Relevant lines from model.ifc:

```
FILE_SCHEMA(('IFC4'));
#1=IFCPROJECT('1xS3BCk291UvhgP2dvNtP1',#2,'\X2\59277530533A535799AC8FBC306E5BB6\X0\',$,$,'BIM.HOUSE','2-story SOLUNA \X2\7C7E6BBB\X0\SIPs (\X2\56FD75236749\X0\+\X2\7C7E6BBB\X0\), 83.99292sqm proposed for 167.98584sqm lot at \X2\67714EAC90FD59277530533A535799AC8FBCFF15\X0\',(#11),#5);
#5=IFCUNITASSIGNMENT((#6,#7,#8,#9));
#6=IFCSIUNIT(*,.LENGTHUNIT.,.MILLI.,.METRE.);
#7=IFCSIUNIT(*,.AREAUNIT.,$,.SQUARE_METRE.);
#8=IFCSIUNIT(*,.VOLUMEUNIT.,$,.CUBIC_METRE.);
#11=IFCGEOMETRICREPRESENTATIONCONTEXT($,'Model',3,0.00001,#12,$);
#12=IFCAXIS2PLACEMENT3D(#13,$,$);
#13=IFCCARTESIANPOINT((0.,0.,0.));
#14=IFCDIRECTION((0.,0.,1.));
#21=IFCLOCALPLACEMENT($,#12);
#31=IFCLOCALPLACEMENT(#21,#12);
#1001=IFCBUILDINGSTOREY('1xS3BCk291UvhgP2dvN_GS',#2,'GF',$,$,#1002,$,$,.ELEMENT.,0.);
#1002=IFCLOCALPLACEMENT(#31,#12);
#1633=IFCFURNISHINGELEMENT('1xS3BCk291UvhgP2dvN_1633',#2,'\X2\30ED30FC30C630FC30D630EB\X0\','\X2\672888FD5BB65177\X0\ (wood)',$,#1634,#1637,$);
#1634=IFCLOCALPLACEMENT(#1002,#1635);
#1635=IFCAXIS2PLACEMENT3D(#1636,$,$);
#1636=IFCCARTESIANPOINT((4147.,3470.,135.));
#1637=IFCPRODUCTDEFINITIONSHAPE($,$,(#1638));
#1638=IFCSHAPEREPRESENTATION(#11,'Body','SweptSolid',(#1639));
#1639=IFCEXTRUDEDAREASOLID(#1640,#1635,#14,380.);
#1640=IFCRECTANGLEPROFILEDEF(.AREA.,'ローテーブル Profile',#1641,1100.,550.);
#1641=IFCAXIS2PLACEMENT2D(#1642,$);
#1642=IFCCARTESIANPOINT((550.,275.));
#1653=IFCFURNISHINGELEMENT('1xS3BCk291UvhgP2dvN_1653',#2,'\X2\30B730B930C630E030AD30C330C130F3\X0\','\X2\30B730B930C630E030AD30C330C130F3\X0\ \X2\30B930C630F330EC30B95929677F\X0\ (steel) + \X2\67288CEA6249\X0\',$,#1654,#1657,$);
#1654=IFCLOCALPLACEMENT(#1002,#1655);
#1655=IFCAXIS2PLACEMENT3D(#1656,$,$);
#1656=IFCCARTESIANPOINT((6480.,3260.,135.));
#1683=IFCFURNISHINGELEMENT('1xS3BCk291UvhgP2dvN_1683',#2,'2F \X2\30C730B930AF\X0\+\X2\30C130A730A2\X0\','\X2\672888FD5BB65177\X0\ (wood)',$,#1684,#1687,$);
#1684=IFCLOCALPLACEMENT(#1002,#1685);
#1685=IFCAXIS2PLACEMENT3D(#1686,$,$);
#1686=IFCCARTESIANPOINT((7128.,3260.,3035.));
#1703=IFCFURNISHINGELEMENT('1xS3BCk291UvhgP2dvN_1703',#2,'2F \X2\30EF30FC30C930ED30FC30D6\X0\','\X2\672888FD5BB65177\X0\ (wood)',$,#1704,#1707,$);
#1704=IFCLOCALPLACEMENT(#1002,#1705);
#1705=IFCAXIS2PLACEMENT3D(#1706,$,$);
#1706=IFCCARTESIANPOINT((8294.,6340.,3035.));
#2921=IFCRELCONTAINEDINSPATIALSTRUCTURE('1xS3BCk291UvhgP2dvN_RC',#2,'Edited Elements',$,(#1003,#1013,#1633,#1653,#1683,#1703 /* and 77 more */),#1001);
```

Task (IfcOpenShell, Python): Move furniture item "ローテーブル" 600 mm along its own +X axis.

```python
import ifcopenshell
import ifcopenshell.api.geometry
import ifcopenshell.util.placement
import ifcopenshell.util.unit

model = ifcopenshell.open("model.ifc")
unit_scale = ifcopenshell.util.unit.calculate_unit_scale(model)

item = model.by_guid("1xS3BCk291UvhgP2dvN_1633")
matrix = ifcopenshell.util.placement.get_local_placement(item.ObjectPlacement)
matrix[:3, 3] += matrix[:3, 0] * 0.6 / unit_scale
ifcopenshell.api.geometry.edit_object_placement(model, product=item, matrix=matrix, is_si=False)

print(ifcopenshell.util.placement.get_local_placement(item.ObjectPlacement).round(3) + 0.0)

model.write("model_v2.ifc")
```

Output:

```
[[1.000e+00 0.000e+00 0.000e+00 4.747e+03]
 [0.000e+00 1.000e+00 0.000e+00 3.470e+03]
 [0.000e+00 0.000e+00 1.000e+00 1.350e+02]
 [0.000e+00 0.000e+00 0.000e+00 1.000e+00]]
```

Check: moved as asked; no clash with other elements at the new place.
